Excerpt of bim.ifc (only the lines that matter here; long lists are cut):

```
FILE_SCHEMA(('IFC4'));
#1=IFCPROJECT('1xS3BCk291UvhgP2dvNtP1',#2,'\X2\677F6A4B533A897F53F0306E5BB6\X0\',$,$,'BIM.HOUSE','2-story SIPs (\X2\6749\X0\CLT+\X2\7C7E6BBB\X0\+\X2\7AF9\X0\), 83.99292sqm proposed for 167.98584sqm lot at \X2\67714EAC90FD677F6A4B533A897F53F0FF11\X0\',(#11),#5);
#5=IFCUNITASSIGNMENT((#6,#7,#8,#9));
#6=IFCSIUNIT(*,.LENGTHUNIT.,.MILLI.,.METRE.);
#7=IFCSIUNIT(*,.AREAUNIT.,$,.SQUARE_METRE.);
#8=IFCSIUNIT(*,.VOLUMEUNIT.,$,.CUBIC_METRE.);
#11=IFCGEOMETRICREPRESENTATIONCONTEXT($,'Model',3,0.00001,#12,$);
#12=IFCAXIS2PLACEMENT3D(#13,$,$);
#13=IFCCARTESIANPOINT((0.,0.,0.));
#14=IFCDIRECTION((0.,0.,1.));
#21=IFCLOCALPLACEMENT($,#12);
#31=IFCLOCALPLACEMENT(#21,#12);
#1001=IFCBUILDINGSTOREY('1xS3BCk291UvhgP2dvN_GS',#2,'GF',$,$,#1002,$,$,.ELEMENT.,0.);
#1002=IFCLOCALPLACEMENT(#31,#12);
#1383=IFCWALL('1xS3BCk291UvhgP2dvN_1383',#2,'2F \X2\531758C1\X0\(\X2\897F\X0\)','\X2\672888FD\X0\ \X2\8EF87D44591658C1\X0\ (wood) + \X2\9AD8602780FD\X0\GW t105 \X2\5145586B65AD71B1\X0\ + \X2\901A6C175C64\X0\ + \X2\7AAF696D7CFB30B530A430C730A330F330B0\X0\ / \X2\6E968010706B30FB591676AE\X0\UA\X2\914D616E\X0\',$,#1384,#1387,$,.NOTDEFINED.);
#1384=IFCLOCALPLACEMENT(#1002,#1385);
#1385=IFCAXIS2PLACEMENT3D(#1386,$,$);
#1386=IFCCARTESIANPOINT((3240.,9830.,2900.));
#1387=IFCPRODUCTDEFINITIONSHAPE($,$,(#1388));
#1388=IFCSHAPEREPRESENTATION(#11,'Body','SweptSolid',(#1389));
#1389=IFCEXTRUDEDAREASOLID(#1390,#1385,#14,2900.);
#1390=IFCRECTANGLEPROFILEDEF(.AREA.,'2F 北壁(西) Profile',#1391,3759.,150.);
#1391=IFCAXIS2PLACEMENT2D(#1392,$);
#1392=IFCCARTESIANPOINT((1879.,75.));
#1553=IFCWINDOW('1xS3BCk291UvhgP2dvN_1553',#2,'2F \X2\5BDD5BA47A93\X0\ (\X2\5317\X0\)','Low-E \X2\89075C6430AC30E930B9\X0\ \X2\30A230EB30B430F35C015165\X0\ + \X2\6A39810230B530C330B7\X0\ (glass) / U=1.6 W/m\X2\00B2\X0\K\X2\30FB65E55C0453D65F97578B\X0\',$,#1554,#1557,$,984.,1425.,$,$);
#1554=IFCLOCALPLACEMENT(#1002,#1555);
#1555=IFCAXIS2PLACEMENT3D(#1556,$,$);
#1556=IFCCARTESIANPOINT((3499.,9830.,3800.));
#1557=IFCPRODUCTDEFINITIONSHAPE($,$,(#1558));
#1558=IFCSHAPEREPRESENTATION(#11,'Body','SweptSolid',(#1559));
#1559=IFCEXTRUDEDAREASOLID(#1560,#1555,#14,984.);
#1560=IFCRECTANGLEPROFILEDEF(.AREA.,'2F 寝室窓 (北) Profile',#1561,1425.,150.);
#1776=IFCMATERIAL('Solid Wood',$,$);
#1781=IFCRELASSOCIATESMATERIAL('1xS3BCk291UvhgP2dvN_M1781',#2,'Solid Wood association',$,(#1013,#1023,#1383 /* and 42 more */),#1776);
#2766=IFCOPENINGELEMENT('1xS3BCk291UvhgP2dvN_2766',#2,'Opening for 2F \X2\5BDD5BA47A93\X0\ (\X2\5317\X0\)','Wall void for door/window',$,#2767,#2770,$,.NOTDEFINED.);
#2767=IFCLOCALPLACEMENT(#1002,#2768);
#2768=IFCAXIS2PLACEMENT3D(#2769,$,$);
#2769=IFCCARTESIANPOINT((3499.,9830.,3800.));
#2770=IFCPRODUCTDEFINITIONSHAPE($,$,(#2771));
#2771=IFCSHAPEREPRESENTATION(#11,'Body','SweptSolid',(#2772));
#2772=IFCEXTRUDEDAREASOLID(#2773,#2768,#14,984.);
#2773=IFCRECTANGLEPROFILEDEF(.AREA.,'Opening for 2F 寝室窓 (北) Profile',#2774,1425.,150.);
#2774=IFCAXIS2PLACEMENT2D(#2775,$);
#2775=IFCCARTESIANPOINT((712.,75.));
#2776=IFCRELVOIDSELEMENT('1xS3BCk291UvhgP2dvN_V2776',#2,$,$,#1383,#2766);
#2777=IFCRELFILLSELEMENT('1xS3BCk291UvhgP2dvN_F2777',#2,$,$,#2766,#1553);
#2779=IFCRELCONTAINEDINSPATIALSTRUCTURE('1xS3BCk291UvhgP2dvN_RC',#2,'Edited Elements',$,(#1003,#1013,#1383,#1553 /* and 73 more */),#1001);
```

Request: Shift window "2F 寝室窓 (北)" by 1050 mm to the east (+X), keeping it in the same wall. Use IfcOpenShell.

```python
import ifcopenshell
import ifcopenshell.api.geometry
import ifcopenshell.util.placement
import ifcopenshell.util.unit

model = ifcopenshell.open("bim.ifc")
unit_scale = ifcopenshell.util.unit.calculate_unit_scale(model)

window = model.by_guid("1xS3BCk291UvhgP2dvN_1553")
opening = window.FillsVoids[0].RelatingOpeningElement
wall = opening.VoidsElements[0].RelatingBuildingElement

wall_matrix = ifcopenshell.util.placement.get_local_placement(wall.ObjectPlacement)
shift = wall_matrix[:3, 0] * 1.05 / unit_scale
before = ifcopenshell.util.placement.get_local_placement(window.ObjectPlacement)[:3, 3].copy()

# The window is not placed relative to its opening, so move both.
for product in (opening, window):
    matrix = ifcopenshell.util.placement.get_local_placement(product.ObjectPlacement)
    matrix[:3, 3] += shift
    ifcopenshell.api.geometry.edit_object_placement(model, product=product, matrix=matrix, is_si=False)

after = ifcopenshell.util.placement.get_local_placement(window.ObjectPlacement)[:3, 3]
print("window moved by", (after - before).round(3) + 0.0)

model.write("bim_updated.ifc")
```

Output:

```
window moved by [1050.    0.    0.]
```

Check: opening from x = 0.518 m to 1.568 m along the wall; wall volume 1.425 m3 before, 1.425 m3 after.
